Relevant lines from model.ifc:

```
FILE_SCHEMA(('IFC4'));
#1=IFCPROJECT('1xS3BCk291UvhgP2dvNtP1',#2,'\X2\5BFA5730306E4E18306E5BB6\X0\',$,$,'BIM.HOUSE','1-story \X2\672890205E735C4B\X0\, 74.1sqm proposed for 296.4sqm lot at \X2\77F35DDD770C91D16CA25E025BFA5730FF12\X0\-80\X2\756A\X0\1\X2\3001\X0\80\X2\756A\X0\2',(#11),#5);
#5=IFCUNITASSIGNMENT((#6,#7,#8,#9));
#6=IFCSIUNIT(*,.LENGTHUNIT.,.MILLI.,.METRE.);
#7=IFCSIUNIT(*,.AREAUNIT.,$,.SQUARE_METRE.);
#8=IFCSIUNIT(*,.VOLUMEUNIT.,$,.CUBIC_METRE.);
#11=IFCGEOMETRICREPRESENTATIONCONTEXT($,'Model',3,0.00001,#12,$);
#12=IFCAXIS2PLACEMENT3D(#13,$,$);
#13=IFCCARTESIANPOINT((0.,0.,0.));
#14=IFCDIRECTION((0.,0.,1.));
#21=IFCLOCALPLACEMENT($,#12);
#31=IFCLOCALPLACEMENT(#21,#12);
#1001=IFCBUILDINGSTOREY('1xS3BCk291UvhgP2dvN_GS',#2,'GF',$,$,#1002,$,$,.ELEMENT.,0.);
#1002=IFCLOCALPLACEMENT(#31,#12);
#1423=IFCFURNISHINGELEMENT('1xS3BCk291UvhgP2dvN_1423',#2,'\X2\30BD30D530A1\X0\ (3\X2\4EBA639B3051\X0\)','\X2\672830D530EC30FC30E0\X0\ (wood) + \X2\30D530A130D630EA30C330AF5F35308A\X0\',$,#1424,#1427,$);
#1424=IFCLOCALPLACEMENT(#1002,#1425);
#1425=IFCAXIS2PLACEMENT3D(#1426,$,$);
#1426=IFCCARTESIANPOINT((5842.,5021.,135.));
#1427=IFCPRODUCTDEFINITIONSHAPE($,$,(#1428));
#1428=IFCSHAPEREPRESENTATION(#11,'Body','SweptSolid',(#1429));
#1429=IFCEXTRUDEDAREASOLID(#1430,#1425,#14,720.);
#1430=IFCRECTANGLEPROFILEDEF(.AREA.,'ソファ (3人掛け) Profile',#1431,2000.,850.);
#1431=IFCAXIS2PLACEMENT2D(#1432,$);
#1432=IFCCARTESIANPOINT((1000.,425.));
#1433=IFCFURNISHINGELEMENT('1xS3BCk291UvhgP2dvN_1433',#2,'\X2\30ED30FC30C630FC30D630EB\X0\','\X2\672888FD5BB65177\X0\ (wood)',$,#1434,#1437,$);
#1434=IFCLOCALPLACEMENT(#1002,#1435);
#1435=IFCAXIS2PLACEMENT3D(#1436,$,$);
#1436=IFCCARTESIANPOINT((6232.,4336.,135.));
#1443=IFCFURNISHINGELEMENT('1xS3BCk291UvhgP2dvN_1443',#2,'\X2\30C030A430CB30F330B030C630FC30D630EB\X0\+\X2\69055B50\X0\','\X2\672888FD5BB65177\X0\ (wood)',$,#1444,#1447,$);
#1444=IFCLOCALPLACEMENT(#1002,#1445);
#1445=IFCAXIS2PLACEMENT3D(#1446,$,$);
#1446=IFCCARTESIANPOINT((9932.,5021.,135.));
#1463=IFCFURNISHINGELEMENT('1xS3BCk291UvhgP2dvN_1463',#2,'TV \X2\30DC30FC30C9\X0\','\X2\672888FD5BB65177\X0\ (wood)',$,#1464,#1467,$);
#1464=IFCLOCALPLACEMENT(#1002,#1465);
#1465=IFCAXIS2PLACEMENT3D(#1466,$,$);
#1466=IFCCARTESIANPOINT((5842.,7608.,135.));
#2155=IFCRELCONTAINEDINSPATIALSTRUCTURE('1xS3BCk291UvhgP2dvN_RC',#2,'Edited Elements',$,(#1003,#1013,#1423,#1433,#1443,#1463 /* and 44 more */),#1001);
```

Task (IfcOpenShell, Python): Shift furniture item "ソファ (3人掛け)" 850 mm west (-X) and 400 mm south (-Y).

```python
import ifcopenshell
import ifcopenshell.api.geometry
import ifcopenshell.util.placement

model = ifcopenshell.open("model.ifc")

item = model.by_guid("1xS3BCk291UvhgP2dvN_1423")
matrix = ifcopenshell.util.placement.get_local_placement(item.ObjectPlacement)
matrix[0, 3] -= 850.0
matrix[1, 3] -= 400.0
ifcopenshell.api.geometry.edit_object_placement(model, product=item, matrix=matrix, is_si=False)

print(ifcopenshell.util.placement.get_local_placement(item.ObjectPlacement).round(3) + 0.0)

model.write("model_updated.ifc")
```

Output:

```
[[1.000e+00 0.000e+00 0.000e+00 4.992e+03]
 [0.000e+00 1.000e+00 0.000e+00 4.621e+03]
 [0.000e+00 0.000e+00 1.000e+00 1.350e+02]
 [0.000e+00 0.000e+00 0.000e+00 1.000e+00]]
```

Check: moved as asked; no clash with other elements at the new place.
